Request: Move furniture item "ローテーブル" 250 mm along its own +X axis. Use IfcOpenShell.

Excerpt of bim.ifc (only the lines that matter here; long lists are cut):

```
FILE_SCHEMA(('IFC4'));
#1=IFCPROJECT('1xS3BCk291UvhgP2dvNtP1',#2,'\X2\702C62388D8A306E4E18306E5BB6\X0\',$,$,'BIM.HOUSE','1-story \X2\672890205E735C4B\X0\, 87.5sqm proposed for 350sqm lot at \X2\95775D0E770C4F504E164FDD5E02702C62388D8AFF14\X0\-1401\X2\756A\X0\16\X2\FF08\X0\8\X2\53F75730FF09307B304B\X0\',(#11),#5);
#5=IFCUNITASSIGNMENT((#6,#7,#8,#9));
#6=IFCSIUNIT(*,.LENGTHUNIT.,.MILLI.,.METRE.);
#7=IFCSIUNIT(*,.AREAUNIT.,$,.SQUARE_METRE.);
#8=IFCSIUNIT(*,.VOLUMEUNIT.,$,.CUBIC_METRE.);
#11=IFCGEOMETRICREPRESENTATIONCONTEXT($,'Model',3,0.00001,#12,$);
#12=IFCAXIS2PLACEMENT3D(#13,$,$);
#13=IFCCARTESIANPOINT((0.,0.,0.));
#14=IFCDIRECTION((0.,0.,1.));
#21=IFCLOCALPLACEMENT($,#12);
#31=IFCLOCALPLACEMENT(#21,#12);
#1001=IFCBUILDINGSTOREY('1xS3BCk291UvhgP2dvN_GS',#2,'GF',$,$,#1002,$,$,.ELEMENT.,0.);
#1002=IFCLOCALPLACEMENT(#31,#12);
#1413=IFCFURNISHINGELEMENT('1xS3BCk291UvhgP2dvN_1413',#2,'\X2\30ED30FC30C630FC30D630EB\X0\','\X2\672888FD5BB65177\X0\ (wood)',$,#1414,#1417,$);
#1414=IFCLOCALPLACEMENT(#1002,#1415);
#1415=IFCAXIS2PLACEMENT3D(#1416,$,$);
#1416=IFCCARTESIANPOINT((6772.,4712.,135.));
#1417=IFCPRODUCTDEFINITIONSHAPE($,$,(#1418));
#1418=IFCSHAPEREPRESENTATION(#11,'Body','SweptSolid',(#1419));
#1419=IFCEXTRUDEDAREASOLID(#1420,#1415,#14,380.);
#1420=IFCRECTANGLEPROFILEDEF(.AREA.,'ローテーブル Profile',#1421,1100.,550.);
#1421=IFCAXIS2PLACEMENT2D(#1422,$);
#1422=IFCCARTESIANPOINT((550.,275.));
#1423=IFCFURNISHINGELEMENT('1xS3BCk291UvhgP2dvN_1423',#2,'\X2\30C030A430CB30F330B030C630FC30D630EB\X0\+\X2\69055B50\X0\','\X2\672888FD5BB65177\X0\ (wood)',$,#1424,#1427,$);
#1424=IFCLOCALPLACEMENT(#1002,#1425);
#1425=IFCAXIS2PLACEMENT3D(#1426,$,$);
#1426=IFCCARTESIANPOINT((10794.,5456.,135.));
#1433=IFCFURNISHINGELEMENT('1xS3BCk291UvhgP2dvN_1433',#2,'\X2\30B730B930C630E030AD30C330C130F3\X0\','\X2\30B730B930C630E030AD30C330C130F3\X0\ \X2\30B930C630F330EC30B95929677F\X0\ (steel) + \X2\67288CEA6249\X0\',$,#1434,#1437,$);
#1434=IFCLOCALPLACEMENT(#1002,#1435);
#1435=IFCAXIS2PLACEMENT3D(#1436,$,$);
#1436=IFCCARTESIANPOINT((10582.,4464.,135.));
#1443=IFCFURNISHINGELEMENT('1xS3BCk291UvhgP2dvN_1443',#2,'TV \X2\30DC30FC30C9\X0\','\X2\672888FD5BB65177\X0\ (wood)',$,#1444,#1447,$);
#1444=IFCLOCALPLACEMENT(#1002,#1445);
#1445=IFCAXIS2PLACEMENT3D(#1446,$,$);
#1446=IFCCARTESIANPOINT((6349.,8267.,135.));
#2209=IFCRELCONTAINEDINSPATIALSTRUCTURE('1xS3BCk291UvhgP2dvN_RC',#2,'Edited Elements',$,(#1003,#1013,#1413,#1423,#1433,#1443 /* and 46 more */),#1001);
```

```python
import ifcopenshell
import ifcopenshell.api.geometry
import ifcopenshell.util.placement

model = ifcopenshell.open("bim.ifc")

item = model.by_id(1413)
matrix = ifcopenshell.util.placement.get_local_placement(item.ObjectPlacement)
matrix[:3, 3] += matrix[:3, 0] * 250.0
ifcopenshell.api.geometry.edit_object_placement(model, product=item, matrix=matrix, is_si=False)

print(ifcopenshell.util.placement.get_local_placement(item.ObjectPlacement).round(3) + 0.0)

model.write("bim_v2.ifc")
```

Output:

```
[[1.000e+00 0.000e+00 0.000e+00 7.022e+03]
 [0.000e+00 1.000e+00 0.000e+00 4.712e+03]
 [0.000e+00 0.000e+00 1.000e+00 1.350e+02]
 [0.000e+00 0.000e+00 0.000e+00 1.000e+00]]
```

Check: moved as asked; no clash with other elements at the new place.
